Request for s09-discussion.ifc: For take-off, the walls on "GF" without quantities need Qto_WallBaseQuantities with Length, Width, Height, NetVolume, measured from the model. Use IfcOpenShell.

First a look at what the model holds.

```python
import ifcopenshell
import ifcopenshell.util.element
import ifcopenshell.util.unit

model = ifcopenshell.open("s09-discussion.ifc")
print(model.schema)
for unit_type in ("LENGTHUNIT", "AREAUNIT", "VOLUMEUNIT"):
    print(unit_type, ifcopenshell.util.unit.calculate_unit_scale(model, unit_type))
storey = next(s for s in model.by_type("IfcBuildingStorey") if s.Name == "GF")
walls = [e for e in ifcopenshell.util.element.get_decomposition(storey) if e.is_a("IfcWall")]
for e in sorted(walls, key=lambda e: e.id()):
    print(e.id(), e.is_a(), e.Name, list(ifcopenshell.util.element.get_psets(e, qtos_only=True)), sep=" | ")
```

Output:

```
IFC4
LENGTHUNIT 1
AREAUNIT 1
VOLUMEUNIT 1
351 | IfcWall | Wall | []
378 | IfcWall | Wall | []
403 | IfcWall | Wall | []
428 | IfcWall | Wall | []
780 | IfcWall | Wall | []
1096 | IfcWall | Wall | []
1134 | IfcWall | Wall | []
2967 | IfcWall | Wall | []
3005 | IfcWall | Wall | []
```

```python
import ifcopenshell
import ifcopenshell.api.pset
import ifcopenshell.geom
import ifcopenshell.util.element
import ifcopenshell.util.shape
import ifcopenshell.util.unit

model = ifcopenshell.open("s09-discussion.ifc")
unit_scale = ifcopenshell.util.unit.calculate_unit_scale(model)
volume_scale = ifcopenshell.util.unit.calculate_unit_scale(model, "VOLUMEUNIT")
settings = ifcopenshell.geom.settings()

storey = next(s for s in model.by_type("IfcBuildingStorey") if s.Name == "GF")
walls = [e for e in ifcopenshell.util.element.get_decomposition(storey) if e.is_a("IfcWall")]

for e in sorted(walls, key=lambda e: e.id()):
    if ifcopenshell.util.element.get_psets(e, qtos_only=True, should_inherit=False):
        continue
    # Geometry comes back in metres, in the element's own axes.
    shape = ifcopenshell.geom.create_shape(settings, e)
    values = {
        "Length": ifcopenshell.util.shape.get_x(shape.geometry) / unit_scale,
        "Width": ifcopenshell.util.shape.get_y(shape.geometry) / unit_scale,
        "Height": ifcopenshell.util.shape.get_z(shape.geometry) / unit_scale,
        "NetVolume": ifcopenshell.util.shape.get_volume(shape.geometry) / volume_scale,
    }
    qto = ifcopenshell.api.pset.add_qto(model, product=e, name="Qto_WallBaseQuantities")
    ifcopenshell.api.pset.edit_qto(model, qto=qto, properties=values)
    print(e.id(), {k: round(v, 3) for k, v in values.items()})

model.write("s09-discussion_v2.ifc")
```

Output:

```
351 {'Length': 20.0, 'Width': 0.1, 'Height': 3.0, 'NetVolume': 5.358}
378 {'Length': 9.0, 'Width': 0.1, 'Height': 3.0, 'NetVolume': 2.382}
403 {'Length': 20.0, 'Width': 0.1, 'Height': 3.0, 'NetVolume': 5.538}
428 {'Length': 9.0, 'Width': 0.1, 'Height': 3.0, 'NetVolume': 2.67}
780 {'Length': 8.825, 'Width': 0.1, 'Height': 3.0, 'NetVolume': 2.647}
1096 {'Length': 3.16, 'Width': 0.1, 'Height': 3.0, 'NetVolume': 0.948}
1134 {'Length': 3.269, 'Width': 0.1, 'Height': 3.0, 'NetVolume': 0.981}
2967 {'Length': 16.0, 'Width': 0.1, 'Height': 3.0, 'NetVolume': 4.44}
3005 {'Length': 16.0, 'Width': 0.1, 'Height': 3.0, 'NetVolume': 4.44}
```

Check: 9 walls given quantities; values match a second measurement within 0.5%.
